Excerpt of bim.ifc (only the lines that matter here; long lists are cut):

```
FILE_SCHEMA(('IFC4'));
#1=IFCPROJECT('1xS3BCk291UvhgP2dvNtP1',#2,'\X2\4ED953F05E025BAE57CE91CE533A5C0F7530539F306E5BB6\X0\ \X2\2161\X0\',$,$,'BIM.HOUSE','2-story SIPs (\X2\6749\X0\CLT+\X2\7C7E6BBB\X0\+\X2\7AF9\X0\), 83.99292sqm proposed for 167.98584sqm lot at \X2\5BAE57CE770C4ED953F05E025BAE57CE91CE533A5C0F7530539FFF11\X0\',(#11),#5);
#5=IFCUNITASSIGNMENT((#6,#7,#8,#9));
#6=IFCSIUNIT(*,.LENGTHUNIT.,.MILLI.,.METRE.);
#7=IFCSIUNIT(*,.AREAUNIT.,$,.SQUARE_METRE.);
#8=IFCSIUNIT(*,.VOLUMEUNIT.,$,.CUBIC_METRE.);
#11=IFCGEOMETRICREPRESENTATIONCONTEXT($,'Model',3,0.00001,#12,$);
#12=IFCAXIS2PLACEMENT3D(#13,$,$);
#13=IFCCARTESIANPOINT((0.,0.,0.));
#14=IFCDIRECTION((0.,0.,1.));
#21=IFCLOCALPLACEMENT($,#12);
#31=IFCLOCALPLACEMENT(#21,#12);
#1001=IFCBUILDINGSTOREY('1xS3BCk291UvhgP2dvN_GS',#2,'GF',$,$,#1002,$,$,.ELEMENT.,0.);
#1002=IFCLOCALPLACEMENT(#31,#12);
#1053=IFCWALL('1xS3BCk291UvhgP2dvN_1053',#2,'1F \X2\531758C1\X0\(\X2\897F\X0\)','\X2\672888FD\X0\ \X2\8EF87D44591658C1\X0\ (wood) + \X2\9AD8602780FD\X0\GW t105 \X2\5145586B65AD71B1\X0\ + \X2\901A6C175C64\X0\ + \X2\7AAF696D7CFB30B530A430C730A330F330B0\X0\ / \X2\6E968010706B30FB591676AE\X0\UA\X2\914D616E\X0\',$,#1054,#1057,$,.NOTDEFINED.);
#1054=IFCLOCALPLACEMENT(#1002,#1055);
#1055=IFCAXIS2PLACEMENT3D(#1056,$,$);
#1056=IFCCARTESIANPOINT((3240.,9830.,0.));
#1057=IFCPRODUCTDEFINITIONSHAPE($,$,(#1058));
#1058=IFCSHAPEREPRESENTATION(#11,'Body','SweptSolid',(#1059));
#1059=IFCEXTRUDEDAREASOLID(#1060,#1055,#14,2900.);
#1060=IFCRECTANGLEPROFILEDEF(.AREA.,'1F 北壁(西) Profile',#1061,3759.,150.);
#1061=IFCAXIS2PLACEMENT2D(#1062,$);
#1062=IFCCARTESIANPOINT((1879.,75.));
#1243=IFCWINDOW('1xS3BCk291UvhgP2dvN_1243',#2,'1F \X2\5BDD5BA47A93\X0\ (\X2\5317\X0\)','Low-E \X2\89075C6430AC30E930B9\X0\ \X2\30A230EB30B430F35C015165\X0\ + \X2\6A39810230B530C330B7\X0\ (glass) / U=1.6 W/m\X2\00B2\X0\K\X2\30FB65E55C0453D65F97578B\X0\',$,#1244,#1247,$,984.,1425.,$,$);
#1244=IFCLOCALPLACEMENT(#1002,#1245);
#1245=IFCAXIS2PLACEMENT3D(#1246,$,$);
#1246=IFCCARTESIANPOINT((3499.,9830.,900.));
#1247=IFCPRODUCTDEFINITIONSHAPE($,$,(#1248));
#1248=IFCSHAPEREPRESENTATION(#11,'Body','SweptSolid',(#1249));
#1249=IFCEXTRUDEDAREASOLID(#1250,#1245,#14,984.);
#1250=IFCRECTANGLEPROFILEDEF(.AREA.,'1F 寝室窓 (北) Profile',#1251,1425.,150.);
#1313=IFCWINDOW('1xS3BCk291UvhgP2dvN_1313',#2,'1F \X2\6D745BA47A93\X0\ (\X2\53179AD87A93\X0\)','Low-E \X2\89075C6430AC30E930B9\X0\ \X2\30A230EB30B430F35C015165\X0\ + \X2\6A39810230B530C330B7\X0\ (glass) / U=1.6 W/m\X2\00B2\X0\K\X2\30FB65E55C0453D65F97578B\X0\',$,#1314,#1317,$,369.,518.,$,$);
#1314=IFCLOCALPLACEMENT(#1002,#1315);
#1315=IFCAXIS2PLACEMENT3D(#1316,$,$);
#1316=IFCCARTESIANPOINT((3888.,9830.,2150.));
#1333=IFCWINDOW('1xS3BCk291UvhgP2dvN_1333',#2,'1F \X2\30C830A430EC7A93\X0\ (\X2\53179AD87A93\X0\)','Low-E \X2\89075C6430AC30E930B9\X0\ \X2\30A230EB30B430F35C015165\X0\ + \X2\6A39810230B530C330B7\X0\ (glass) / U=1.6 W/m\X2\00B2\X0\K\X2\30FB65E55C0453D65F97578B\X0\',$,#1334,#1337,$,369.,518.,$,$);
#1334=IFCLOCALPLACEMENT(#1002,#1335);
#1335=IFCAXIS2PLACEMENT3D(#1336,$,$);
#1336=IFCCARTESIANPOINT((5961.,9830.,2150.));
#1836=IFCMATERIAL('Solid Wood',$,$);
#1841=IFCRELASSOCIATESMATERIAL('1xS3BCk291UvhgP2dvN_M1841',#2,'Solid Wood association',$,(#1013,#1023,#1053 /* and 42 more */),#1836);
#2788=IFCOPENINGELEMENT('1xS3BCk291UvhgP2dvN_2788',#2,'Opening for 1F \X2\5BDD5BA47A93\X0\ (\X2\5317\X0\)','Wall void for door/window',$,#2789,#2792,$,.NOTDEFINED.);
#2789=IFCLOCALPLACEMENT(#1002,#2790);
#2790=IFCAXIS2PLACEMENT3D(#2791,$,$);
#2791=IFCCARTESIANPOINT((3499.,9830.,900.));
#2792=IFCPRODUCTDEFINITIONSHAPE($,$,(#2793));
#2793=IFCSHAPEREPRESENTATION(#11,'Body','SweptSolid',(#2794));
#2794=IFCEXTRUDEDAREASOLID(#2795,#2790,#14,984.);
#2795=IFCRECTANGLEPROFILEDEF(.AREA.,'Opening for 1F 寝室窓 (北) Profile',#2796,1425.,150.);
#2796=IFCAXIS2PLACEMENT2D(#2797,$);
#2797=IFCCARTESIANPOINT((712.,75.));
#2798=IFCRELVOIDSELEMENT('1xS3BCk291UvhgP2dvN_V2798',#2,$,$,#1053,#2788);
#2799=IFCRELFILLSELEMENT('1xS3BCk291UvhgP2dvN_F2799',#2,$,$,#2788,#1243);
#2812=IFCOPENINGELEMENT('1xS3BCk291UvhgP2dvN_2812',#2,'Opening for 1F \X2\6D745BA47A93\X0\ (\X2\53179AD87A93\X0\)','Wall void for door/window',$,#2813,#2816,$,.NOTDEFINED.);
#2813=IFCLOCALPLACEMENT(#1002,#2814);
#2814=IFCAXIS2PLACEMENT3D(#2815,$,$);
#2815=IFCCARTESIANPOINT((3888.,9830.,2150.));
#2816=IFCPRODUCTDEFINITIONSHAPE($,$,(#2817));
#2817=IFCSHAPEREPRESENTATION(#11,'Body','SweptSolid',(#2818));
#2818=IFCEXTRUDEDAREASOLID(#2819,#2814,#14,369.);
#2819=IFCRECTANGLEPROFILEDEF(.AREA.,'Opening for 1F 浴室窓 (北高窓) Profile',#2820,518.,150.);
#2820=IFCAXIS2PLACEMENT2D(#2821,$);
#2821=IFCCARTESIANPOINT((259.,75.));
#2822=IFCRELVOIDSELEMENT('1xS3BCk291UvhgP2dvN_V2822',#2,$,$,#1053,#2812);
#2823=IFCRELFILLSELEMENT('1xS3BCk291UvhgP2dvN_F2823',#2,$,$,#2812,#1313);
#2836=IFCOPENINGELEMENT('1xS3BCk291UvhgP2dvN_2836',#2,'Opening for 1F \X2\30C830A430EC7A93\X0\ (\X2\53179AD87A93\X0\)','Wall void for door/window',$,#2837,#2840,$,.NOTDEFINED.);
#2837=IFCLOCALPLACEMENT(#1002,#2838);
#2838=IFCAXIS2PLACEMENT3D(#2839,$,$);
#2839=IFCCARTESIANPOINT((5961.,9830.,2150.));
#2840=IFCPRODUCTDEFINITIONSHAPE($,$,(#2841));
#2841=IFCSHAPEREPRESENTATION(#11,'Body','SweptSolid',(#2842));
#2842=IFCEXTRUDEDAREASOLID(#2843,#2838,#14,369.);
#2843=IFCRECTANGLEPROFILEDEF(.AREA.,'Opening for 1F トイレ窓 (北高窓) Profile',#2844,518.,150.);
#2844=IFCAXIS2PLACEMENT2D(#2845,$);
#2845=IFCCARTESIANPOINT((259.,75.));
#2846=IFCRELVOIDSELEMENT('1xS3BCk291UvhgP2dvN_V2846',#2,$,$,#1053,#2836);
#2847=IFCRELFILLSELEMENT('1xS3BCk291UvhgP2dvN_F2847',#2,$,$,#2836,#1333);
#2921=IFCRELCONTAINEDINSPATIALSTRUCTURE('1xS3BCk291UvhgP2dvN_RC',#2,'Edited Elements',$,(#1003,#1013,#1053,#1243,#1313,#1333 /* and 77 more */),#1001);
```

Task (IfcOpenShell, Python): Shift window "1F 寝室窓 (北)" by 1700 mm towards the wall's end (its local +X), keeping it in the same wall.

```python
import ifcopenshell
import ifcopenshell.api.geometry
import ifcopenshell.util.placement

model = ifcopenshell.open("bim.ifc")

window = model.by_id(1243)
opening = window.FillsVoids[0].RelatingOpeningElement
wall = opening.VoidsElements[0].RelatingBuildingElement

wall_matrix = ifcopenshell.util.placement.get_local_placement(wall.ObjectPlacement)
shift = wall_matrix[:3, 0] * 1700.0
before = ifcopenshell.util.placement.get_local_placement(window.ObjectPlacement)[:3, 3].copy()

# The window is not placed relative to its opening, so move both.
for product in (opening, window):
    matrix = ifcopenshell.util.placement.get_local_placement(product.ObjectPlacement)
    matrix[:3, 3] += shift
    ifcopenshell.api.geometry.edit_object_placement(model, product=product, matrix=matrix, is_si=False)

after = ifcopenshell.util.placement.get_local_placement(window.ObjectPlacement)[:3, 3]
print("window moved by", (after - before).round(3) + 0.0)

model.write("bim-out.ifc")
```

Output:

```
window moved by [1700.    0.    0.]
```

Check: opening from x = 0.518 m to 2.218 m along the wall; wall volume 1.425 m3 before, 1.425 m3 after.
